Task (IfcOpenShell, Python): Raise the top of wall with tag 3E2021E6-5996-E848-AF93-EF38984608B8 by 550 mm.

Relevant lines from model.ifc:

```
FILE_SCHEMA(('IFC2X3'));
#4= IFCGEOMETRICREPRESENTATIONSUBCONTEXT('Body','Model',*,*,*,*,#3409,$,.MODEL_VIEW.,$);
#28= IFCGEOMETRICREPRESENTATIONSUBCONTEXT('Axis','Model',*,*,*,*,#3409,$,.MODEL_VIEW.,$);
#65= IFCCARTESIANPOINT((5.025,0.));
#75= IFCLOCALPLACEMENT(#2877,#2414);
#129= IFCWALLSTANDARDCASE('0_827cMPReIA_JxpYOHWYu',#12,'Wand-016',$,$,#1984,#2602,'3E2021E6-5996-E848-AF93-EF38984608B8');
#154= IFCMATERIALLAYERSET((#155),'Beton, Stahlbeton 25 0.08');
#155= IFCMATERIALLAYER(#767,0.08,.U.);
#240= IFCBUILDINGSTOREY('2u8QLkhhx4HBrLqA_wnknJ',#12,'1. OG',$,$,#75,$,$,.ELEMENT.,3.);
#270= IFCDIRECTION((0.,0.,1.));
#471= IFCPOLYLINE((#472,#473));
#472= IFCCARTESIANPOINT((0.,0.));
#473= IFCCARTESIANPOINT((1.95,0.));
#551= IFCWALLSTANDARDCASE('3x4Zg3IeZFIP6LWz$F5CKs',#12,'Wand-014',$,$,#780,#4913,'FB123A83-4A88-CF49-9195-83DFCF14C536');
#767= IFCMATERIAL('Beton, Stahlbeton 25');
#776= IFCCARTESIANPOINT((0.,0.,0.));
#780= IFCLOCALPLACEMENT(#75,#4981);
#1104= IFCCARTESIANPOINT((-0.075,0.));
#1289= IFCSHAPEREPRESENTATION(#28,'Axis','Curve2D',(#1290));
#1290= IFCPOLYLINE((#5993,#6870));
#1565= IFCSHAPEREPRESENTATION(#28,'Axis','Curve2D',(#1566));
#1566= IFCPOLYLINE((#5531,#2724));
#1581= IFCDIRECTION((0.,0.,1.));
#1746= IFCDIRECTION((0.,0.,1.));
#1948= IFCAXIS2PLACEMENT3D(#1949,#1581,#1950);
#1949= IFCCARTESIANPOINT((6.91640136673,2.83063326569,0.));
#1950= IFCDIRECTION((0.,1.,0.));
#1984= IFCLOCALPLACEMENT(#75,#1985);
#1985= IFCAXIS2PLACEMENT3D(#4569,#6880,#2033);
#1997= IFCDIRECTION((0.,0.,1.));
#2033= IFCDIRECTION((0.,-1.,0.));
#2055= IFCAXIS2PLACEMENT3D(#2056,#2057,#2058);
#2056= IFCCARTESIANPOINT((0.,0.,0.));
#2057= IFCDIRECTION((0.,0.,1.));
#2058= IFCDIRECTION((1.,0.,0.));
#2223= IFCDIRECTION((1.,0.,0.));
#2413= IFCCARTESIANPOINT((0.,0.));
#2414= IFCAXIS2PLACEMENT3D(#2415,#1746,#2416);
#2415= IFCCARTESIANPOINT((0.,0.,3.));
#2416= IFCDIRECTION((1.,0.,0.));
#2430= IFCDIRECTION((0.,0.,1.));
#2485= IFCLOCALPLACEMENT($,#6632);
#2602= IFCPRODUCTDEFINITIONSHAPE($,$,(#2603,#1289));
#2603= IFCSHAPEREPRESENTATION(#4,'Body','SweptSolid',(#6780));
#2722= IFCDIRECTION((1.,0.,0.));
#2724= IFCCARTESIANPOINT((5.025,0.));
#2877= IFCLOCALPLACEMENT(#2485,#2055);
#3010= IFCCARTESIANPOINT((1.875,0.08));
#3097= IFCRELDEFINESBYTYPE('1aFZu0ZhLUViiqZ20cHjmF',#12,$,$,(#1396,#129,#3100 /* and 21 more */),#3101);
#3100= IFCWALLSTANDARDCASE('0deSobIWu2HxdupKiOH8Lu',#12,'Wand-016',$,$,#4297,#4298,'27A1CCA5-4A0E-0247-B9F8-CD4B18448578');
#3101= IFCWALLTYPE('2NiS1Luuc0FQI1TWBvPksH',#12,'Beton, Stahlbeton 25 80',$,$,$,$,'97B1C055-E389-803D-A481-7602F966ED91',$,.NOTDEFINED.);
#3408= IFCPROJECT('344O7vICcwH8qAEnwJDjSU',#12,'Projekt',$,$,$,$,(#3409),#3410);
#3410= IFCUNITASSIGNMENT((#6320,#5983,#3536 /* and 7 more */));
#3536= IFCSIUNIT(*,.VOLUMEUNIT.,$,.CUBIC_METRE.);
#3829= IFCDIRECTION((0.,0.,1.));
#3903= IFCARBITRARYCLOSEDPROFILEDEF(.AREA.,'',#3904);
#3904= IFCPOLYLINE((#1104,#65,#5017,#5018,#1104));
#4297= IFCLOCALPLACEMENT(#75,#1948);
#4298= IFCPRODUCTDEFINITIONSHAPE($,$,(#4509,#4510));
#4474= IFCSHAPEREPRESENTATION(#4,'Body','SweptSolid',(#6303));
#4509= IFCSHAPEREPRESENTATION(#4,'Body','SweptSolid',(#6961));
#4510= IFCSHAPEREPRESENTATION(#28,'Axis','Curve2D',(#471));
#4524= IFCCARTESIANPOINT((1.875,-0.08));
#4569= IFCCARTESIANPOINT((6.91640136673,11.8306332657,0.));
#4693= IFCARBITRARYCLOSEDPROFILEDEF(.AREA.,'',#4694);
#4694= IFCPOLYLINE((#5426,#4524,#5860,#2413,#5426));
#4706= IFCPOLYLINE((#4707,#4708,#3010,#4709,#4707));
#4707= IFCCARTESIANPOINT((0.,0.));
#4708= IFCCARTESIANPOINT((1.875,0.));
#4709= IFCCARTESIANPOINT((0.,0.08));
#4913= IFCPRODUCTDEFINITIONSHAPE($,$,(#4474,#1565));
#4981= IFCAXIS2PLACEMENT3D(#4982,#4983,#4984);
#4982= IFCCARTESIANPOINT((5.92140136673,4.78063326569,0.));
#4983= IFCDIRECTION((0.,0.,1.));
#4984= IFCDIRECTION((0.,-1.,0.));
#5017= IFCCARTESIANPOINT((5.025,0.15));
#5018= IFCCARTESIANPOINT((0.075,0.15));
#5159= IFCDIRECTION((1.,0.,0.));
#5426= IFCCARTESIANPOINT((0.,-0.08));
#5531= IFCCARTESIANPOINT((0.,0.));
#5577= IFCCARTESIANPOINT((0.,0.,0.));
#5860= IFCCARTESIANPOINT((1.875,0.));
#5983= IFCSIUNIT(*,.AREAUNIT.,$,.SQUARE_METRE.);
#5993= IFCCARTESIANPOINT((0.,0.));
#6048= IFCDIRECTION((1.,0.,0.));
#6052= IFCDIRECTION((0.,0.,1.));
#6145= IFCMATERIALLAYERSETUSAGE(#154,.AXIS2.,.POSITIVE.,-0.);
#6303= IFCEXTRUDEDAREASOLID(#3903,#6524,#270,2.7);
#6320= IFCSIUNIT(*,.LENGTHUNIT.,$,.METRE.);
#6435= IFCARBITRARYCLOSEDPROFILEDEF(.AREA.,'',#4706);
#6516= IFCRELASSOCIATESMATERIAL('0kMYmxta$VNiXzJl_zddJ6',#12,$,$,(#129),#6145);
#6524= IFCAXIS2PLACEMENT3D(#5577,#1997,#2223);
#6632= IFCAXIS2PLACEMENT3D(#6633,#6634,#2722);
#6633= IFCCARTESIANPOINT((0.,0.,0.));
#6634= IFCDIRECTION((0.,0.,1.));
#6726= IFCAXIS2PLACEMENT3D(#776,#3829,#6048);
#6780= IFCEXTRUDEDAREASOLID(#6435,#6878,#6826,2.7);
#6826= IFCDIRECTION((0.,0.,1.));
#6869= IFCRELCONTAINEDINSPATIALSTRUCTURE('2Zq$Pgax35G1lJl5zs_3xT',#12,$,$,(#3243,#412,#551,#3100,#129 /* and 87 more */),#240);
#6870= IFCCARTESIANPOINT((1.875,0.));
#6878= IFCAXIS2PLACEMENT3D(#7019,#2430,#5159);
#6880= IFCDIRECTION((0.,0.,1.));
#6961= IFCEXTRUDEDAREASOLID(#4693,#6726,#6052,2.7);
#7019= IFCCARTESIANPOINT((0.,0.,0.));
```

```python
import ifcopenshell
import ifcopenshell.geom
import ifcopenshell.util.representation
import ifcopenshell.util.shape

model = ifcopenshell.open("model.ifc")
settings = ifcopenshell.geom.settings()


def volume(element):
    """Net volume in cubic metres, openings subtracted."""
    shape = ifcopenshell.geom.create_shape(settings, element)
    return ifcopenshell.util.shape.get_volume(shape.geometry)


wall = model.by_guid("0_827cMPReIA_JxpYOHWYu")
before = volume(wall)

body = ifcopenshell.util.representation.get_representation(wall, "Model", "Body")
solid = body.Items[0]
old_height = solid.Depth
solid.Depth += 0.55
after = volume(wall)

print(f"height {old_height:g} -> {solid.Depth:g}, volume {before:.3f} -> {after:.3f} m3")

model.write("model_rev.ifc")
```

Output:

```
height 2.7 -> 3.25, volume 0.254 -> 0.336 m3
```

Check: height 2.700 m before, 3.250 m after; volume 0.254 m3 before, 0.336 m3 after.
